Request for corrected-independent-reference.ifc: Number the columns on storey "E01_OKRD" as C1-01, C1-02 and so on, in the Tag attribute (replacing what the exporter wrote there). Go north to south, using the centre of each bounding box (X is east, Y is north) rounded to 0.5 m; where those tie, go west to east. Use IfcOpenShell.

First a look at what the model holds.

```python
import ifcopenshell
import ifcopenshell.util.element
import ifcopenshell.util.placement

model = ifcopenshell.open("corrected-independent-reference.ifc")
print(model.schema)
storey = next(s for s in model.by_type("IfcBuildingStorey") if s.Name == "E01_OKRD")
columns = [e for e in ifcopenshell.util.element.get_decomposition(storey) if e.is_a("IfcColumn")]
for e in sorted(columns, key=lambda e: e.id()):
    origin = ifcopenshell.util.placement.get_local_placement(e.ObjectPlacement)[:3, 3]
    print(e.id(), e.Tag, e.Name, origin.round(2) + 0.0, sep=" | ")
```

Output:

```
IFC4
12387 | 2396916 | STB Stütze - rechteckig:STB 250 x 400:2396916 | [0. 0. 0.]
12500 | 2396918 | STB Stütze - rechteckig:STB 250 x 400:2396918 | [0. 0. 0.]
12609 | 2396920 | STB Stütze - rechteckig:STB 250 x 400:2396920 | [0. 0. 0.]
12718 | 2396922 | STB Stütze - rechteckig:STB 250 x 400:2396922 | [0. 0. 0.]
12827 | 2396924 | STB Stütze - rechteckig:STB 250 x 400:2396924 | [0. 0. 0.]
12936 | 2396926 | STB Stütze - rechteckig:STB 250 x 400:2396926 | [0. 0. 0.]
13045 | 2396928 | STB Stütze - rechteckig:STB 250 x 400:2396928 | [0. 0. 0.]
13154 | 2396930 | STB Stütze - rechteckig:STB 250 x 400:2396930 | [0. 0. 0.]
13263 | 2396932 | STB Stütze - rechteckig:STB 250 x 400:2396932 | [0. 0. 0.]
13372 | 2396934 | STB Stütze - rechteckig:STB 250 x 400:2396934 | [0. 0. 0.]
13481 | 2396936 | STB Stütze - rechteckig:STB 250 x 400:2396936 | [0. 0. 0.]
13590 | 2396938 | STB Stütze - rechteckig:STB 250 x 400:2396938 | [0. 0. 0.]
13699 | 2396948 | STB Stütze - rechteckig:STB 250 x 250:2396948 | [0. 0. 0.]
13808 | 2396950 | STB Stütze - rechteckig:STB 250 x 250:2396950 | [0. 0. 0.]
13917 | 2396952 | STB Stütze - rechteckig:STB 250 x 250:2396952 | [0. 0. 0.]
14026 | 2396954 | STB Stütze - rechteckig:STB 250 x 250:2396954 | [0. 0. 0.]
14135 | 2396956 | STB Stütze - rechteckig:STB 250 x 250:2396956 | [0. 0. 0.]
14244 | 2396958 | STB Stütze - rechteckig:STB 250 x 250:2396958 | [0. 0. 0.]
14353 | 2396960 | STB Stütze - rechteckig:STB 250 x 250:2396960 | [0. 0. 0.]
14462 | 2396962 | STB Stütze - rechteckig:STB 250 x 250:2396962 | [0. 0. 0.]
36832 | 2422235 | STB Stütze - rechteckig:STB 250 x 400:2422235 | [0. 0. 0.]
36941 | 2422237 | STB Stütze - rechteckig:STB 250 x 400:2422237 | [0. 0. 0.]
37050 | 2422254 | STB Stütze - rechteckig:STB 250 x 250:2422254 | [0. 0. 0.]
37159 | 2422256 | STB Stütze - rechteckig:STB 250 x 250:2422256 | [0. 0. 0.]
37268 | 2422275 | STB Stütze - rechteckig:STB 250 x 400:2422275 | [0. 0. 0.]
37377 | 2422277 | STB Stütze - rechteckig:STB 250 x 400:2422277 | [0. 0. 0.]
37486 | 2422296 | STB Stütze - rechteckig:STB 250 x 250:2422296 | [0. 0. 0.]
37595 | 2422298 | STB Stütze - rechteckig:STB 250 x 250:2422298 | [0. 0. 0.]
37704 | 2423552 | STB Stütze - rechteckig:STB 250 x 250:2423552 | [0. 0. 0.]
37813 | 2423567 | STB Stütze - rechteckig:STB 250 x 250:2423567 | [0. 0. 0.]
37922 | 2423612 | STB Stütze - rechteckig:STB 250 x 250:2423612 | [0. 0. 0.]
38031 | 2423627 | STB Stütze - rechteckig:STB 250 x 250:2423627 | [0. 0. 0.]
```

```python
import ifcopenshell
import ifcopenshell.geom
import ifcopenshell.util.element
import ifcopenshell.util.shape

model = ifcopenshell.open("corrected-independent-reference.ifc")
settings = ifcopenshell.geom.settings()
settings.set("use-world-coords", True)


def centre(element):
    shape = ifcopenshell.geom.create_shape(settings, element)
    return ifcopenshell.util.shape.get_bbox_centroid(shape.geometry)


storey = next(s for s in model.by_type("IfcBuildingStorey") if s.Name == "E01_OKRD")
columns = [e for e in ifcopenshell.util.element.get_decomposition(storey) if e.is_a("IfcColumn")]

# Insertion points can sit at a corner or the storey origin, so sort by the geometry (in metres).
centres = {e: centre(e) for e in columns}
columns.sort(key=lambda e: (-round(centres[e][1] / 0.5), centres[e][0]))

for i, e in enumerate(columns, start=1):
    number = f"C1-{i:02d}"
    e.Tag = number
    print(e.id(), number)

model.write("corrected-independent-reference_updated.ifc")
```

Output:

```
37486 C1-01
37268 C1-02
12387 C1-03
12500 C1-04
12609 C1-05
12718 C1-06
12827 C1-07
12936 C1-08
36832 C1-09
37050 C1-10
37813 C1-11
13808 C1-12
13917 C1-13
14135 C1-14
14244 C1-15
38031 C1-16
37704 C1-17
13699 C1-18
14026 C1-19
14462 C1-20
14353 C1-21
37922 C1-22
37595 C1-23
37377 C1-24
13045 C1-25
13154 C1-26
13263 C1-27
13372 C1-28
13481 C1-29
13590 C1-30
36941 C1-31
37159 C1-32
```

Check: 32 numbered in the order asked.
